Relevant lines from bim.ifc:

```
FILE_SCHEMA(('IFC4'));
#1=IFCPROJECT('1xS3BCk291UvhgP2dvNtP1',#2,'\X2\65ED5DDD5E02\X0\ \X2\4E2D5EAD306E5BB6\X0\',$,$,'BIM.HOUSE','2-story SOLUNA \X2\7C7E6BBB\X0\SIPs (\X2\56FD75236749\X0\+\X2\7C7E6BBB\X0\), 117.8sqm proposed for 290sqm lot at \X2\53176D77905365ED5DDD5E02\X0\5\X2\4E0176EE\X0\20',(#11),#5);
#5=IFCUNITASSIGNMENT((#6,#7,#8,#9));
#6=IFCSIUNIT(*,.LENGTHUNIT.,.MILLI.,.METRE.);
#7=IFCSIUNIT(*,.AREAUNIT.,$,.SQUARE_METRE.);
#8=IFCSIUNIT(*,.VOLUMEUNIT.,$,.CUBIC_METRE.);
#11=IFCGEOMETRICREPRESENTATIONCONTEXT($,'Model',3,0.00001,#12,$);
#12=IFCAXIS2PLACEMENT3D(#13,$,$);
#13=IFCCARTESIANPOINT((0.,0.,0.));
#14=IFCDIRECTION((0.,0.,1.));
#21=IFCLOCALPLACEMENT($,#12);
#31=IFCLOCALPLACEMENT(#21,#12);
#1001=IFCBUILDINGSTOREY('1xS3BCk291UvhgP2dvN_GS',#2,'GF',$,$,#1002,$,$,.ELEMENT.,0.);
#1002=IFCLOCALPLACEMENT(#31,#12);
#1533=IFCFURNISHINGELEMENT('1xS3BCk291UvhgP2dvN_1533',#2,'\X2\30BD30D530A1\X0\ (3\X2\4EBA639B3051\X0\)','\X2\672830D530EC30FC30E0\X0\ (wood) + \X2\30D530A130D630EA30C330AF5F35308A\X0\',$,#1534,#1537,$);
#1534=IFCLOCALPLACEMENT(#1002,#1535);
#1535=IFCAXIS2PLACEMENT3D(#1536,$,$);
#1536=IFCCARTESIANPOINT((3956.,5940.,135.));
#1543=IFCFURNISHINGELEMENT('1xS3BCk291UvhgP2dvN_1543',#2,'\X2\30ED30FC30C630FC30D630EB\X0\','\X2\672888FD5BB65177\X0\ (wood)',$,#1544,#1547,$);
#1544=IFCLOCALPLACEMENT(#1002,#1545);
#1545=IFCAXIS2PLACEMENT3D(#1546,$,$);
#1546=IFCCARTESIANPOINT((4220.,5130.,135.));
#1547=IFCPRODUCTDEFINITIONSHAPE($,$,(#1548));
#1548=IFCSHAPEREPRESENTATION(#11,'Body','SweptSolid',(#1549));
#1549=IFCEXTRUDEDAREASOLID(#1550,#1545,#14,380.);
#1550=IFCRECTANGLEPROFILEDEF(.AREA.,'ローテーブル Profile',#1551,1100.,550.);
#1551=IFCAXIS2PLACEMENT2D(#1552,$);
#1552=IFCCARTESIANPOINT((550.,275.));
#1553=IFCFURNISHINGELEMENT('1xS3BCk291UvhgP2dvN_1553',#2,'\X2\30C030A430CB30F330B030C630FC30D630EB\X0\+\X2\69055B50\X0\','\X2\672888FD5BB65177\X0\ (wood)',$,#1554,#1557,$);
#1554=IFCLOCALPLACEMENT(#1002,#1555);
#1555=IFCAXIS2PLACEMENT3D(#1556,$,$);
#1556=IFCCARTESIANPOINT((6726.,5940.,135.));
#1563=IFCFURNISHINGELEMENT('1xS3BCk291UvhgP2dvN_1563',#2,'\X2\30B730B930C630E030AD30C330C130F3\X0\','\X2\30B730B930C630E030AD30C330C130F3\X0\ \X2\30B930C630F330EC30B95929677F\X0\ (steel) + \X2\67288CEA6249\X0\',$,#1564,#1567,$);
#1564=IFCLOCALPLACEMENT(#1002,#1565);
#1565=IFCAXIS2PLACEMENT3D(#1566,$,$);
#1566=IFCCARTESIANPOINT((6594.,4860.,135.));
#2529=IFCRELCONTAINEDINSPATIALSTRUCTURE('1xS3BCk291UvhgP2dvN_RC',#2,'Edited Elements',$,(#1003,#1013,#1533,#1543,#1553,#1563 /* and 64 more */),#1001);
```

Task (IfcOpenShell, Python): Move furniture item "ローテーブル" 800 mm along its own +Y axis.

```python
import ifcopenshell
import ifcopenshell.api.geometry
import ifcopenshell.util.placement
import ifcopenshell.util.unit

model = ifcopenshell.open("bim.ifc")
unit_scale = ifcopenshell.util.unit.calculate_unit_scale(model)

item = model.by_guid("1xS3BCk291UvhgP2dvN_1543")
matrix = ifcopenshell.util.placement.get_local_placement(item.ObjectPlacement)
matrix[:3, 3] += matrix[:3, 1] * 0.8 / unit_scale
ifcopenshell.api.geometry.edit_object_placement(model, product=item, matrix=matrix, is_si=False)

print(ifcopenshell.util.placement.get_local_placement(item.ObjectPlacement).round(3) + 0.0)

model.write("bim-out.ifc")
```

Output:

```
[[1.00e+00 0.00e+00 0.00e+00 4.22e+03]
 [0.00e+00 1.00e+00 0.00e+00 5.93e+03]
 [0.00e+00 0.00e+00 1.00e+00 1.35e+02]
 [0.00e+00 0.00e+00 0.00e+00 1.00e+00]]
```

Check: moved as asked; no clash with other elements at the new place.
